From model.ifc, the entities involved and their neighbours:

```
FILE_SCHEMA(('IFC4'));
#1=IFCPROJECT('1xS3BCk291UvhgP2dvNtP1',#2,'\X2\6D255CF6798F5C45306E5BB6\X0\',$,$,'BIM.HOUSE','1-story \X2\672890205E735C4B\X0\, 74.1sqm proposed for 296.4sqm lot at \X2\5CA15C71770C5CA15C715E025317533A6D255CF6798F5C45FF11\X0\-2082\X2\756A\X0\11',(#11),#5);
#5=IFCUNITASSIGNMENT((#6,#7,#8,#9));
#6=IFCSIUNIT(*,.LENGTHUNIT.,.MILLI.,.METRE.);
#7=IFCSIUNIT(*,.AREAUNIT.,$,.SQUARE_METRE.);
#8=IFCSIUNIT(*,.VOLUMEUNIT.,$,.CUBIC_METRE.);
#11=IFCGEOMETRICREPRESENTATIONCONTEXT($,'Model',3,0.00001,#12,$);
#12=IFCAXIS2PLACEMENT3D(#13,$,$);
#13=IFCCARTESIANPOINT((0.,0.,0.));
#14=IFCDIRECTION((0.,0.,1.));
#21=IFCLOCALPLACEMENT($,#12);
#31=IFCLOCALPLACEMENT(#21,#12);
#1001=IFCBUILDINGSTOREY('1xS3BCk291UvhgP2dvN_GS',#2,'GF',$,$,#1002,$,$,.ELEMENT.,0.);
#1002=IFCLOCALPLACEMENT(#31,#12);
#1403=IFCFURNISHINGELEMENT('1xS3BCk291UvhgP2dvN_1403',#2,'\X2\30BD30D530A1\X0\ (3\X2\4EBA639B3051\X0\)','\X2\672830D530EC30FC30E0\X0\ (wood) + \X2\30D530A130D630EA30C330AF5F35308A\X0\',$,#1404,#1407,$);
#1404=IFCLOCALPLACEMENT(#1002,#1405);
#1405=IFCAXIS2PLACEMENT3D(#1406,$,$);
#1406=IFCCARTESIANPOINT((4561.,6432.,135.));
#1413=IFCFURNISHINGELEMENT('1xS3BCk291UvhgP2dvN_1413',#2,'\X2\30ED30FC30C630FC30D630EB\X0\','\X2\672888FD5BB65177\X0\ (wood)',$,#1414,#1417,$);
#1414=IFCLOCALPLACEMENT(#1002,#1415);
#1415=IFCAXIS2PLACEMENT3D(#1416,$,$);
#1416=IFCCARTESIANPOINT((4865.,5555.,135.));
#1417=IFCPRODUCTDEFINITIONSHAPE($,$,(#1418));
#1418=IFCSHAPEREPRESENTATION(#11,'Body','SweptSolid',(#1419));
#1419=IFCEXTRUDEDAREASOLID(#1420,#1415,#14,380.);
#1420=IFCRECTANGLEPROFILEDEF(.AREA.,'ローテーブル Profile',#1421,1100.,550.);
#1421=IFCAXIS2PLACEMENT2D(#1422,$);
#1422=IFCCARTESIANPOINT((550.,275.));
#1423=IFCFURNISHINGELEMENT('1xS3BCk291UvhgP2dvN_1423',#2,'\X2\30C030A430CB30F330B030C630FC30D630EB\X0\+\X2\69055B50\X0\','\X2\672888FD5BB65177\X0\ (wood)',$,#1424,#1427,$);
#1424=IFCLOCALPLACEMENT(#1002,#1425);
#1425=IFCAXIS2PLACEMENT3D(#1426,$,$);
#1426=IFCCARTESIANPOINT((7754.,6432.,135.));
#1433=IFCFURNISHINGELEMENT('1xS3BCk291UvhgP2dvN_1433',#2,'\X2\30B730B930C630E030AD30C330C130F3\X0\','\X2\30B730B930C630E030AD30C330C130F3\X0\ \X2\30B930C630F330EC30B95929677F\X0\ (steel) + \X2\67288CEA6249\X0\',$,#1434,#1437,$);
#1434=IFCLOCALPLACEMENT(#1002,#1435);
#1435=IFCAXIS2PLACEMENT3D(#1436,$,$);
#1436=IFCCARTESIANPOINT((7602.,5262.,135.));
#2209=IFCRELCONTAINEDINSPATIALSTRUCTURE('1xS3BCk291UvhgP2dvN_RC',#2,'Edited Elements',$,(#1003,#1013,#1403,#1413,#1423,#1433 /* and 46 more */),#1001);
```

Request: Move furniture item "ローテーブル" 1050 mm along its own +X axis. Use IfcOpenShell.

```python
import ifcopenshell
import ifcopenshell.api.geometry
import ifcopenshell.util.placement
import ifcopenshell.util.unit

model = ifcopenshell.open("model.ifc")
unit_scale = ifcopenshell.util.unit.calculate_unit_scale(model)

item = model.by_guid("1xS3BCk291UvhgP2dvN_1413")
matrix = ifcopenshell.util.placement.get_local_placement(item.ObjectPlacement)
matrix[:3, 3] += matrix[:3, 0] * 1.05 / unit_scale
ifcopenshell.api.geometry.edit_object_placement(model, product=item, matrix=matrix, is_si=False)

print(ifcopenshell.util.placement.get_local_placement(item.ObjectPlacement).round(3) + 0.0)

model.write("model_rev.ifc")
```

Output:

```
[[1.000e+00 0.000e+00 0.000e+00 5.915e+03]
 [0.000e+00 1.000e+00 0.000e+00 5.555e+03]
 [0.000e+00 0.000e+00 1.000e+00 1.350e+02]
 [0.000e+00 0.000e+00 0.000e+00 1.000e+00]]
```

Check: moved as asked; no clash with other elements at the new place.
